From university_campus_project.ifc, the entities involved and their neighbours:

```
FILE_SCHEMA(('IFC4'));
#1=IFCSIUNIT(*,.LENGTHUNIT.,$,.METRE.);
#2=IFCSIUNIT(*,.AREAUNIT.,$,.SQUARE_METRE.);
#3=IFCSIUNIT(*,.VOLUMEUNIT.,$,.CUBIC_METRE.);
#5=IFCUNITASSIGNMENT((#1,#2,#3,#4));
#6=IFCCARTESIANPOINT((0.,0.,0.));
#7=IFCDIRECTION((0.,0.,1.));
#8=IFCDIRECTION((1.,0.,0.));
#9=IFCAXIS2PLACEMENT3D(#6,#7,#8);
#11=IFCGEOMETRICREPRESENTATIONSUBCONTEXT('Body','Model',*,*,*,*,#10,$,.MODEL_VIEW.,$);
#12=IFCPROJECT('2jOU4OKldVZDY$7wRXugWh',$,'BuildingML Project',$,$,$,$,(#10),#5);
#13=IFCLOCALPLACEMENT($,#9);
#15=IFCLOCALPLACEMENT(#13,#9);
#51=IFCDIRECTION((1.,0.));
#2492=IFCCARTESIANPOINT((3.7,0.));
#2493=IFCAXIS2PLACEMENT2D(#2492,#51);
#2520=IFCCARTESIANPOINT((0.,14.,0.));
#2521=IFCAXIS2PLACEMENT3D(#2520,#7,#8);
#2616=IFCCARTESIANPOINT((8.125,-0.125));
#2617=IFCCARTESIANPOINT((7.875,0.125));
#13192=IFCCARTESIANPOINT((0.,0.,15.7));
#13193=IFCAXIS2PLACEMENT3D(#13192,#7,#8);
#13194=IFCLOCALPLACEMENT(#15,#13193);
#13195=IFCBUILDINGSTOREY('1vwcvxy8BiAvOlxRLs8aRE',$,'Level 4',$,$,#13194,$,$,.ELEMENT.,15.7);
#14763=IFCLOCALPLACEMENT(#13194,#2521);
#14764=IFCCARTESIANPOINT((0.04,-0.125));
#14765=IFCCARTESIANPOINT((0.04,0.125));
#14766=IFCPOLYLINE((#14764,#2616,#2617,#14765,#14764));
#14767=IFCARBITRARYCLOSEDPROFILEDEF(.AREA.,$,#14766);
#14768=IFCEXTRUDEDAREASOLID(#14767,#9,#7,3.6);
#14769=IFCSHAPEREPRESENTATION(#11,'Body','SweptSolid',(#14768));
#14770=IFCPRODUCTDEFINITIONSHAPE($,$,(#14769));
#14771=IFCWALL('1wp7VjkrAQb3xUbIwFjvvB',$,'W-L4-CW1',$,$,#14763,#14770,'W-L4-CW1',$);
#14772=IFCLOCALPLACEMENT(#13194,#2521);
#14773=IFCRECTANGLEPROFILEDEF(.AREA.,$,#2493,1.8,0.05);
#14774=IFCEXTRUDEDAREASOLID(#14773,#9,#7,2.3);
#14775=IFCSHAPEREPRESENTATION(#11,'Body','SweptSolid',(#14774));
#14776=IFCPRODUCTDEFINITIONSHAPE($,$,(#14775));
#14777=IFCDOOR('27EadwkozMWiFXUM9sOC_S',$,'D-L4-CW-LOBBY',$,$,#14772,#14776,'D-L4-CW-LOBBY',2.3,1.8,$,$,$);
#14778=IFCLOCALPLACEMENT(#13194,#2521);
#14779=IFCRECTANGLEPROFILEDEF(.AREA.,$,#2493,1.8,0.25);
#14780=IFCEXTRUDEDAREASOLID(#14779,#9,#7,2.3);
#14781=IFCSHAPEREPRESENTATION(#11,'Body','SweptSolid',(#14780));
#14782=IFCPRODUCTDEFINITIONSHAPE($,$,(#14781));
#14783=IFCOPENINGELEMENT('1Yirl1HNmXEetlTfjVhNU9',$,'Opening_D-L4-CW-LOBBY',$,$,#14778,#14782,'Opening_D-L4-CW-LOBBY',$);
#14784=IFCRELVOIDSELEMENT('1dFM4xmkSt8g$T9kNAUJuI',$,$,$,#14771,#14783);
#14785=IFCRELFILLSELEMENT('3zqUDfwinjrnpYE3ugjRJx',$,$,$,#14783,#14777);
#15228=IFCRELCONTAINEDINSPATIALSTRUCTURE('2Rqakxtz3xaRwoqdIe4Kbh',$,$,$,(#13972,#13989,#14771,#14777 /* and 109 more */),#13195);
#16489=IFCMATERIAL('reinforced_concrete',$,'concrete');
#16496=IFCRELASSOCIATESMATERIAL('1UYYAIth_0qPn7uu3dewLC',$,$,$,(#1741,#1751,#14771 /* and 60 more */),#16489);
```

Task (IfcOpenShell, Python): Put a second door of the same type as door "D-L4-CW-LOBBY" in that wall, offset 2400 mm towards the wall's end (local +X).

```python
import ifcopenshell
import ifcopenshell.api.feature
import ifcopenshell.api.geometry
import ifcopenshell.api.root
import ifcopenshell.geom
import ifcopenshell.util.element
import ifcopenshell.util.placement
import ifcopenshell.util.shape

model = ifcopenshell.open("university_campus_project.ifc")
settings = ifcopenshell.geom.settings()


def volume(element):
    """Net volume in cubic metres, openings subtracted."""
    shape = ifcopenshell.geom.create_shape(settings, element)
    return ifcopenshell.util.shape.get_volume(shape.geometry)


door = model.by_guid("27EadwkozMWiFXUM9sOC_S")
opening = door.FillsVoids[0].RelatingOpeningElement
wall = opening.VoidsElements[0].RelatingBuildingElement
before = volume(wall)
shift = ifcopenshell.util.placement.get_local_placement(wall.ObjectPlacement)[:3, 0] * 2.4

# copy_class copies the void relationship, type, container and properties, but no geometry.
new_opening = ifcopenshell.api.root.copy_class(model, product=opening)
new_opening.Representation = ifcopenshell.util.element.copy_deep(
    model, opening.Representation, exclude=["IfcGeometricRepresentationContext", "IfcRepresentationMap"]
)
new_opening.Tag = None
new_door = ifcopenshell.api.root.copy_class(model, product=door)
new_door.Representation = ifcopenshell.util.element.copy_deep(
    model, door.Representation, exclude=["IfcGeometricRepresentationContext", "IfcRepresentationMap"]
)
new_door.Tag = None
ifcopenshell.api.feature.add_filling(model, opening=new_opening, element=new_door)

for old, new in ((opening, new_opening), (door, new_door)):
    matrix = ifcopenshell.util.placement.get_local_placement(old.ObjectPlacement)
    matrix[:3, 3] += shift
    ifcopenshell.api.geometry.edit_object_placement(model, product=new, matrix=matrix, is_si=False)

after = volume(wall)

print(f"wall volume {before:.3f} -> {after:.3f} m3")

model.write("university_campus_project-out.ifc")
```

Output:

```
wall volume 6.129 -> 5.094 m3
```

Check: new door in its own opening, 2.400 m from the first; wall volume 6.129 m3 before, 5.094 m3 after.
